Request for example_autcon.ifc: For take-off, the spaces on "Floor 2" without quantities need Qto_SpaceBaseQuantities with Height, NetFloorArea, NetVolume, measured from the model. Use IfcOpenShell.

First a look at what the model holds.

```python
import ifcopenshell
import ifcopenshell.util.element
import ifcopenshell.util.unit

model = ifcopenshell.open("example_autcon.ifc")
print(model.schema)
for unit_type in ("LENGTHUNIT", "AREAUNIT", "VOLUMEUNIT"):
    print(unit_type, ifcopenshell.util.unit.calculate_unit_scale(model, unit_type))
storey = next(s for s in model.by_type("IfcBuildingStorey") if s.Name == "Floor 2")
spaces = [e for e in ifcopenshell.util.element.get_decomposition(storey) if e.is_a("IfcSpace")]
for e in sorted(spaces, key=lambda e: e.id()):
    print(e.id(), e.is_a(), e.Name, list(ifcopenshell.util.element.get_psets(e, qtos_only=True)), sep=" | ")
```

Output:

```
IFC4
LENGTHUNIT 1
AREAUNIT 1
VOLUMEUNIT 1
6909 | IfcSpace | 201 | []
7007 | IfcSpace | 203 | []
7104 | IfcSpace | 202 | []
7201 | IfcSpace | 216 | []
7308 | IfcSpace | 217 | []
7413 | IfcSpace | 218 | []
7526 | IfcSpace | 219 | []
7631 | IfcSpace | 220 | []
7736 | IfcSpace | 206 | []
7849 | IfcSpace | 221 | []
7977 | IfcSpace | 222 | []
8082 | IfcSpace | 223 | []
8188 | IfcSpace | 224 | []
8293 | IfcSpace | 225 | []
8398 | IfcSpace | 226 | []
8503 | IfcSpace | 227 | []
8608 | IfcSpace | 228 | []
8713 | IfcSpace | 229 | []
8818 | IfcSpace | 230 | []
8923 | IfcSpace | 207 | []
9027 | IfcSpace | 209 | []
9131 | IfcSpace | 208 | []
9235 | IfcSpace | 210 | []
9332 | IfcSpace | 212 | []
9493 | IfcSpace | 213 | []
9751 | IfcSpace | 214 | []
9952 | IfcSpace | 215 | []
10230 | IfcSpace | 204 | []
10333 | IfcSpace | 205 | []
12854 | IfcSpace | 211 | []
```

```python
import ifcopenshell
import ifcopenshell.api.pset
import ifcopenshell.geom
import ifcopenshell.util.element
import ifcopenshell.util.shape
import ifcopenshell.util.unit

model = ifcopenshell.open("example_autcon.ifc")
unit_scale = ifcopenshell.util.unit.calculate_unit_scale(model)
area_scale = ifcopenshell.util.unit.calculate_unit_scale(model, "AREAUNIT")
volume_scale = ifcopenshell.util.unit.calculate_unit_scale(model, "VOLUMEUNIT")
settings = ifcopenshell.geom.settings()

storey = next(s for s in model.by_type("IfcBuildingStorey") if s.Name == "Floor 2")
spaces = [e for e in ifcopenshell.util.element.get_decomposition(storey) if e.is_a("IfcSpace")]

for e in sorted(spaces, key=lambda e: e.id()):
    if ifcopenshell.util.element.get_psets(e, qtos_only=True, should_inherit=False):
        continue
    # Geometry comes back in metres, in the element's own axes.
    shape = ifcopenshell.geom.create_shape(settings, e)
    values = {
        "Height": ifcopenshell.util.shape.get_z(shape.geometry) / unit_scale,
        "NetFloorArea": ifcopenshell.util.shape.get_footprint_area(shape.geometry) / area_scale,
        "NetVolume": ifcopenshell.util.shape.get_volume(shape.geometry) / volume_scale,
    }
    qto = ifcopenshell.api.pset.add_qto(model, product=e, name="Qto_SpaceBaseQuantities")
    ifcopenshell.api.pset.edit_qto(model, qto=qto, properties=values)
    print(e.id(), {k: round(v, 3) for k, v in values.items()})

model.write("example_autcon_edited.ifc")
```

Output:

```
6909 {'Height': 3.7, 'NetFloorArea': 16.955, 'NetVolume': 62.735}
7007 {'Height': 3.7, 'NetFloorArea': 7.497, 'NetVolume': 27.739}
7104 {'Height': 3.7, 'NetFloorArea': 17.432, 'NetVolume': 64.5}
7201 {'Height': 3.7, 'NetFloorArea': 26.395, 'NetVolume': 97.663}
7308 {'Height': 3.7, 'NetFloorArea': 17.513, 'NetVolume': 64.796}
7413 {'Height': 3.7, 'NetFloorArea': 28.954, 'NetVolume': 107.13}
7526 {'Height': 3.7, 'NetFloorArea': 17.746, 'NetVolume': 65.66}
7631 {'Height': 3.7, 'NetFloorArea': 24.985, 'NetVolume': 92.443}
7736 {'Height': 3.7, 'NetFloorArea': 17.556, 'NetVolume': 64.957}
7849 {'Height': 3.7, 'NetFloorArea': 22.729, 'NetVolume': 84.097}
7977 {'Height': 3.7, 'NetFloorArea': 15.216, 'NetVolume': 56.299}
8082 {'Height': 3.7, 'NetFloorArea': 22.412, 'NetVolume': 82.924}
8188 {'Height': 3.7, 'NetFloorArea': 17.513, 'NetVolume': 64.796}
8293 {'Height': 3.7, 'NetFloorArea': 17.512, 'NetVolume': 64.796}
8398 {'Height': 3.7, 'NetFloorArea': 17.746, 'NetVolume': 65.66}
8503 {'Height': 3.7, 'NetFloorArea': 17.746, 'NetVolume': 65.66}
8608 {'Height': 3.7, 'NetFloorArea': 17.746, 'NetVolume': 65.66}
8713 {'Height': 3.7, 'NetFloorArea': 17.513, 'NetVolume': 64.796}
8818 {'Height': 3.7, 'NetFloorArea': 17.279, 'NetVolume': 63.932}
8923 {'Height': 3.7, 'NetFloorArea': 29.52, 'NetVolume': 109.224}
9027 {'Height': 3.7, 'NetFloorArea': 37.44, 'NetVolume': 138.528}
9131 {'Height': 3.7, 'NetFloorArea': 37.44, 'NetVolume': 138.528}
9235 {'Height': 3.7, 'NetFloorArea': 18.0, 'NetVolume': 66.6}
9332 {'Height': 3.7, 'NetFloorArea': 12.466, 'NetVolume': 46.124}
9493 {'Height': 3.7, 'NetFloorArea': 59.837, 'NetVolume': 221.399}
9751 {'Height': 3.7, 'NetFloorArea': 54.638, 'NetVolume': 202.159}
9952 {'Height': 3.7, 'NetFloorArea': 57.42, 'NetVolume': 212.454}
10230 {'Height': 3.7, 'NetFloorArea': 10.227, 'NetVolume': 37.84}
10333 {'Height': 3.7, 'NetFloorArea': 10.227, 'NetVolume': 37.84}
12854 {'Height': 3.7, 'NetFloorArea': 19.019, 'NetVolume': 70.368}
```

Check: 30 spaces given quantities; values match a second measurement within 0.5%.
